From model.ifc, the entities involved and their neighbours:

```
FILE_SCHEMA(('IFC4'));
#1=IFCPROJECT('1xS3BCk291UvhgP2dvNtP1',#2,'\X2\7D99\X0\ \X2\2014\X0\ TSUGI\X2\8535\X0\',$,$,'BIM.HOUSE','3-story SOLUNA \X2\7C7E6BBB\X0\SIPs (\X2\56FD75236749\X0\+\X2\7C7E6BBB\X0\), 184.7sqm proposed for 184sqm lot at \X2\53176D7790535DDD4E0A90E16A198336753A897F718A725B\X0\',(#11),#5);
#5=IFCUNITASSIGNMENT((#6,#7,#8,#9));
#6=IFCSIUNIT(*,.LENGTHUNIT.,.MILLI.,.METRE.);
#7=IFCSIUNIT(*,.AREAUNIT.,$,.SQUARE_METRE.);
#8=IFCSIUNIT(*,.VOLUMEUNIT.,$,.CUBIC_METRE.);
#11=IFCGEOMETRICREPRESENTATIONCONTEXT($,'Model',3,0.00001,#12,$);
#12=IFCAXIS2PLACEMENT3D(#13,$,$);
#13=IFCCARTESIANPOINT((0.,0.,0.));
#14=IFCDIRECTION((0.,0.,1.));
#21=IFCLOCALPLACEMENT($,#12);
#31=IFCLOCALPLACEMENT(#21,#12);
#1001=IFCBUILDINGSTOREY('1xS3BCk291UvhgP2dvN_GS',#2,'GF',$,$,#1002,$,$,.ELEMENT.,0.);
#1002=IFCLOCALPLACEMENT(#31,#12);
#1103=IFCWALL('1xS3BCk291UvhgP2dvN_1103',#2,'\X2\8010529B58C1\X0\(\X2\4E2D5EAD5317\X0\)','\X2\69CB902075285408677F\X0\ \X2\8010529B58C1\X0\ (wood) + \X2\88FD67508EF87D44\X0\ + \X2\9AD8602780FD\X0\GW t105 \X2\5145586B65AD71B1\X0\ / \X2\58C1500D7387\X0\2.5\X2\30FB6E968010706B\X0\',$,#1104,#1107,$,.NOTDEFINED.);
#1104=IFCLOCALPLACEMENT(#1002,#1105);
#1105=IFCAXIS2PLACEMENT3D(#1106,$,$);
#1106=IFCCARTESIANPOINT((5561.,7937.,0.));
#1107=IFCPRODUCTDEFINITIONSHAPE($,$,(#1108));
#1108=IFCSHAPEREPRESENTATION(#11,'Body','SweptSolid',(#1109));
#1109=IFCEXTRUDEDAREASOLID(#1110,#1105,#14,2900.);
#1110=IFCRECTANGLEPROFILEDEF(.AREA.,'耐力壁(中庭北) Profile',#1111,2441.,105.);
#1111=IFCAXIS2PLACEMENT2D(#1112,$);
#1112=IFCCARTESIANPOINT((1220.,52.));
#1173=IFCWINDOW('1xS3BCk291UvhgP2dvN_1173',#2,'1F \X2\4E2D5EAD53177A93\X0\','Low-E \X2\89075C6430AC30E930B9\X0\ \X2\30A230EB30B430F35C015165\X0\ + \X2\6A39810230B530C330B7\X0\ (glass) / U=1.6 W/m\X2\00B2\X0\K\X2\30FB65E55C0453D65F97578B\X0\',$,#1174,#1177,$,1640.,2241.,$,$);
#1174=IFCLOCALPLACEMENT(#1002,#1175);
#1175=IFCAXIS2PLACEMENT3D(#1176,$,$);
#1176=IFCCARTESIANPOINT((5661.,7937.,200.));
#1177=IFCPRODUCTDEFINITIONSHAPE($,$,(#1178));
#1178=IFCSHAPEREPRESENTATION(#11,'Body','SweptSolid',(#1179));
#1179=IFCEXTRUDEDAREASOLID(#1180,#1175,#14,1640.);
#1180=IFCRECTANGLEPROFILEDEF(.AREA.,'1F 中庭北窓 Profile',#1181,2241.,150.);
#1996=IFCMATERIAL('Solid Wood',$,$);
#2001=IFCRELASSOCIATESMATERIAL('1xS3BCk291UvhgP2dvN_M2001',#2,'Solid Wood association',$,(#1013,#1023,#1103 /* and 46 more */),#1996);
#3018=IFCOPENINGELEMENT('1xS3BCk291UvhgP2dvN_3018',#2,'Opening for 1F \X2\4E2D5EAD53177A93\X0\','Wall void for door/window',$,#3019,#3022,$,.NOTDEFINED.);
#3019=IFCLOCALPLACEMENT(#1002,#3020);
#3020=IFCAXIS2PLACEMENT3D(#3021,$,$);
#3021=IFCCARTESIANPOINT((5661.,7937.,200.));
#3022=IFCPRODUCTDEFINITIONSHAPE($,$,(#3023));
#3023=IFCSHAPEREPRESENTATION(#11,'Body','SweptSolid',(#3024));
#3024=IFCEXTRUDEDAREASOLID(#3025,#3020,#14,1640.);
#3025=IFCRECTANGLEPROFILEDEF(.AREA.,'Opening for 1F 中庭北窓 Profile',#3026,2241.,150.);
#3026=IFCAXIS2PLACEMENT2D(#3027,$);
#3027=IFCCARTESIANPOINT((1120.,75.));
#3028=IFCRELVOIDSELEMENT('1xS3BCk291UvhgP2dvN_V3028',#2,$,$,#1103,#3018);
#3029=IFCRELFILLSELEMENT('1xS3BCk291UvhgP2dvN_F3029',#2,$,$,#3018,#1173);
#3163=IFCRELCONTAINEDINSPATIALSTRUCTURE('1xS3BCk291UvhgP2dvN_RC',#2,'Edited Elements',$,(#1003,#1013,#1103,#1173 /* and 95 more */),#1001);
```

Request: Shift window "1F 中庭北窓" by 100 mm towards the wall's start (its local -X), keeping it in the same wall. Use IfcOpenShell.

```python
import ifcopenshell
import ifcopenshell.api.geometry
import ifcopenshell.util.placement
import ifcopenshell.util.unit

model = ifcopenshell.open("model.ifc")
unit_scale = ifcopenshell.util.unit.calculate_unit_scale(model)

window = model.by_guid("1xS3BCk291UvhgP2dvN_1173")
opening = window.FillsVoids[0].RelatingOpeningElement
wall = opening.VoidsElements[0].RelatingBuildingElement

wall_matrix = ifcopenshell.util.placement.get_local_placement(wall.ObjectPlacement)
shift = wall_matrix[:3, 0] * -0.1 / unit_scale
before = ifcopenshell.util.placement.get_local_placement(window.ObjectPlacement)[:3, 3].copy()

# The window is not placed relative to its opening, so move both.
for product in (opening, window):
    matrix = ifcopenshell.util.placement.get_local_placement(product.ObjectPlacement)
    matrix[:3, 3] += shift
    ifcopenshell.api.geometry.edit_object_placement(model, product=product, matrix=matrix, is_si=False)

after = ifcopenshell.util.placement.get_local_placement(window.ObjectPlacement)[:3, 3]
print("window moved by", (after - before).round(3) + 0.0)

model.write("model_updated.ifc")
```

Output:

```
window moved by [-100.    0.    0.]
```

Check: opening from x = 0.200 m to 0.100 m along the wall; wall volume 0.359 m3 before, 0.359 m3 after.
